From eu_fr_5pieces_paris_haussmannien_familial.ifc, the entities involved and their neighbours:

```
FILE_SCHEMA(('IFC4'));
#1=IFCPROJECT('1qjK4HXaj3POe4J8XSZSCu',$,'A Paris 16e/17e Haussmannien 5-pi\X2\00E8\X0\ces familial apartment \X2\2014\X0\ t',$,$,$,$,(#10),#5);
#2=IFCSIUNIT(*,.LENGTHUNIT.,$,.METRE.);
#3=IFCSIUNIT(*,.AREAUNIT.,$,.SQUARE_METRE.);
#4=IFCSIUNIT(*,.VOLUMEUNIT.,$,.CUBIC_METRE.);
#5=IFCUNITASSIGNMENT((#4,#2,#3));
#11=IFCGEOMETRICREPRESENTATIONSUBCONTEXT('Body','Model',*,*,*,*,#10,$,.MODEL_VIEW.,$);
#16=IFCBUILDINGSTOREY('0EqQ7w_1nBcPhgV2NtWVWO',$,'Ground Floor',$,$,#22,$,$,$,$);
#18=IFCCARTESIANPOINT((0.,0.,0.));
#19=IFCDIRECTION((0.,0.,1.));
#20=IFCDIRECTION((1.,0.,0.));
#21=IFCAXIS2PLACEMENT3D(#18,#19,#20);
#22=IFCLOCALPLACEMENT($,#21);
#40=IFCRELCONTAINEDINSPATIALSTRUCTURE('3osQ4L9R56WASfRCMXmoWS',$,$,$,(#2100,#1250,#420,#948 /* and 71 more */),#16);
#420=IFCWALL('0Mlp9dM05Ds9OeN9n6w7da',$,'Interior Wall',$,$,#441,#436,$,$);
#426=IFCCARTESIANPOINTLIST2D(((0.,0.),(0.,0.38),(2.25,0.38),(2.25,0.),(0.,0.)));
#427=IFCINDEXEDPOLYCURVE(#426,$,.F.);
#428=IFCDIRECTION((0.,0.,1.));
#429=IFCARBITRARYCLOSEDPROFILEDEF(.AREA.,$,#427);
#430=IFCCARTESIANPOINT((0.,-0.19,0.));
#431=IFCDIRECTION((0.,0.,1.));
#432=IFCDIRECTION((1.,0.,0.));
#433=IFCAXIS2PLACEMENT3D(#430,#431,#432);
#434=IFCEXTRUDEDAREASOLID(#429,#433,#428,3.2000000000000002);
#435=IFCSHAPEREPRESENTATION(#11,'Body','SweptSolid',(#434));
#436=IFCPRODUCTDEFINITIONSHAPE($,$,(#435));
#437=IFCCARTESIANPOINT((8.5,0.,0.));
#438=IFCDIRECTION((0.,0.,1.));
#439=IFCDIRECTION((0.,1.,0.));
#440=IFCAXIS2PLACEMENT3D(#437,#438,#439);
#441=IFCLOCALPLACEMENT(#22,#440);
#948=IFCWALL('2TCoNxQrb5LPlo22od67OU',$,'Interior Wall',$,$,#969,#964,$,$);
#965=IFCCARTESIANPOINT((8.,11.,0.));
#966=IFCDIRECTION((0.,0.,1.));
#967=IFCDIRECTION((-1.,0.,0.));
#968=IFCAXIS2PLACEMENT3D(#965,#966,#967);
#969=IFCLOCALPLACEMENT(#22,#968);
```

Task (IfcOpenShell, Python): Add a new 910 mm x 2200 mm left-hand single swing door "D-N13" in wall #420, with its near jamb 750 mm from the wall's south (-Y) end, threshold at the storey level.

```python
import numpy as np
import ifcopenshell
import ifcopenshell.api.feature
import ifcopenshell.api.geometry
import ifcopenshell.api.root
import ifcopenshell.api.spatial
import ifcopenshell.geom
import ifcopenshell.util.element
import ifcopenshell.util.placement
import ifcopenshell.util.representation
import ifcopenshell.util.shape
import ifcopenshell.util.unit

model = ifcopenshell.open("eu_fr_5pieces_paris_haussmannien_familial.ifc")
unit_scale = ifcopenshell.util.unit.calculate_unit_scale(model)
settings = ifcopenshell.geom.settings()


def volume(element):
    """Net volume in cubic metres, openings subtracted."""
    shape = ifcopenshell.geom.create_shape(settings, element)
    return ifcopenshell.util.shape.get_volume(shape.geometry)


wall = model.by_guid("0Mlp9dM05Ds9OeN9n6w7da")
storey = ifcopenshell.util.element.get_container(wall, ifc_class="IfcBuildingStorey")
context = ifcopenshell.util.representation.get_context(model, "Model", "Body", "MODEL_VIEW")
before = volume(wall)

width, height, from_end, sill = 0.91, 2.2, 0.75, 0.0  # metres

# The wall runs along its own X axis, and the end named is its -X end.
wall_shape = ifcopenshell.geom.create_shape(settings, wall)
x, y, z = ifcopenshell.util.shape.get_vertices(wall_shape.geometry).T
start = x.min() + from_end
face, thickness = float(y.min()), float(y.max() - y.min())
wall_matrix = ifcopenshell.util.placement.get_local_placement(wall.ObjectPlacement)
level = ifcopenshell.util.placement.get_local_placement(storey.ObjectPlacement)[2, 3]


def in_wall(x, y):
    """Placement at x, y metres in the wall's axes, at sill height."""
    matrix = wall_matrix.copy()
    matrix[:, 3] = wall_matrix @ np.array([x / unit_scale, y / unit_scale, 0.0, 1.0])
    matrix[2, 3] = level + sill / unit_scale
    return matrix


# Opening: a box that overshoots both wall faces by 50 mm.
opening = ifcopenshell.api.root.create_entity(model, ifc_class="IfcOpeningElement", predefined_type="OPENING")
box = ifcopenshell.api.geometry.add_wall_representation(
    model, context=context, length=width, height=height, thickness=thickness + 0.1
)
ifcopenshell.api.geometry.assign_representation(model, product=opening, representation=box)
ifcopenshell.api.geometry.edit_object_placement(model, product=opening, matrix=in_wall(start, face - 0.05), is_si=False)
ifcopenshell.api.feature.add_feature(model, feature=opening, element=wall)

door = ifcopenshell.api.root.create_entity(model, ifc_class="IfcDoor", name="D-N13", predefined_type="DOOR")
door.OverallWidth, door.OverallHeight = width / unit_scale, height / unit_scale
door.OperationType = "SINGLE_SWING_LEFT"
body = ifcopenshell.api.geometry.add_door_representation(
    model,
    context=context,
    overall_width=door.OverallWidth,
    overall_height=door.OverallHeight,
    operation_type="SINGLE_SWING_LEFT",
    lining_properties={"LiningDepth": thickness / unit_scale, "ThresholdDepth": thickness / unit_scale},
)
ifcopenshell.api.geometry.assign_representation(model, product=door, representation=body)
ifcopenshell.api.spatial.assign_container(model, products=[door], relating_structure=storey)
ifcopenshell.api.feature.add_filling(model, opening=opening, element=door)

# The lining spans the wall, so the door starts at the wall face.
ifcopenshell.api.geometry.edit_object_placement(model, product=door, matrix=in_wall(start, face), is_si=False)

after = volume(wall)

print(f"wall volume {before:.3f} -> {after:.3f} m3")

model.write("eu_fr_5pieces_paris_haussmannien_familial-out.ifc")
```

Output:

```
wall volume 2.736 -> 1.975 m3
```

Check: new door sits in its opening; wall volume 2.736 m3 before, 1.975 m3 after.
